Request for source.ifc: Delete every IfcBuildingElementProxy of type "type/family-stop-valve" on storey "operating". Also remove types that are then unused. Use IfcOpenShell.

First a look at what the model holds.

```python
import ifcopenshell
import ifcopenshell.util.element

model = ifcopenshell.open("source.ifc")
print(model.schema)
storey = next(s for s in model.by_type("IfcBuildingStorey") if s.Name == "operating")
proxies = [e for e in ifcopenshell.util.element.get_decomposition(storey) if e.is_a("IfcBuildingElementProxy")]
seen = {}
for e in proxies:
    element_type = ifcopenshell.util.element.get_type(e)
    name = element_type.Name if element_type not in (None, e) else None
    seen[name] = seen.get(name, 0) + 1
for name, count in sorted(seen.items(), key=str):
    print(count, "x", name)
```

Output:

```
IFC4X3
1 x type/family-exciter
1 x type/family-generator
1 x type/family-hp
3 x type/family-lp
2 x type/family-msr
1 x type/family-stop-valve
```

```python
import ifcopenshell
import ifcopenshell.api.root
import ifcopenshell.util.element

model = ifcopenshell.open("source.ifc")

storey = next(s for s in model.by_type("IfcBuildingStorey") if s.Name == "operating")
proxies = [e for e in ifcopenshell.util.element.get_decomposition(storey) if e.is_a("IfcBuildingElementProxy")]
targets = [e for e in proxies if (t := ifcopenshell.util.element.get_type(e)) not in (None, e) and t.Name == "type/family-stop-valve"]
types = {ifcopenshell.util.element.get_type(e) for e in targets} - {None, *targets}

for e in targets:
    ifcopenshell.api.root.remove_product(model, product=e)
print(len(targets), "removed")

unused = [t for t in types if not ifcopenshell.util.element.get_types(t)]
for t in unused:
    ifcopenshell.api.root.remove_product(model, product=t)
print(len(unused), "unused types removed")

model.write("source_edited.ifc")
```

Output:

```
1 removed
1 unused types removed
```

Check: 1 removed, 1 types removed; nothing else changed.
